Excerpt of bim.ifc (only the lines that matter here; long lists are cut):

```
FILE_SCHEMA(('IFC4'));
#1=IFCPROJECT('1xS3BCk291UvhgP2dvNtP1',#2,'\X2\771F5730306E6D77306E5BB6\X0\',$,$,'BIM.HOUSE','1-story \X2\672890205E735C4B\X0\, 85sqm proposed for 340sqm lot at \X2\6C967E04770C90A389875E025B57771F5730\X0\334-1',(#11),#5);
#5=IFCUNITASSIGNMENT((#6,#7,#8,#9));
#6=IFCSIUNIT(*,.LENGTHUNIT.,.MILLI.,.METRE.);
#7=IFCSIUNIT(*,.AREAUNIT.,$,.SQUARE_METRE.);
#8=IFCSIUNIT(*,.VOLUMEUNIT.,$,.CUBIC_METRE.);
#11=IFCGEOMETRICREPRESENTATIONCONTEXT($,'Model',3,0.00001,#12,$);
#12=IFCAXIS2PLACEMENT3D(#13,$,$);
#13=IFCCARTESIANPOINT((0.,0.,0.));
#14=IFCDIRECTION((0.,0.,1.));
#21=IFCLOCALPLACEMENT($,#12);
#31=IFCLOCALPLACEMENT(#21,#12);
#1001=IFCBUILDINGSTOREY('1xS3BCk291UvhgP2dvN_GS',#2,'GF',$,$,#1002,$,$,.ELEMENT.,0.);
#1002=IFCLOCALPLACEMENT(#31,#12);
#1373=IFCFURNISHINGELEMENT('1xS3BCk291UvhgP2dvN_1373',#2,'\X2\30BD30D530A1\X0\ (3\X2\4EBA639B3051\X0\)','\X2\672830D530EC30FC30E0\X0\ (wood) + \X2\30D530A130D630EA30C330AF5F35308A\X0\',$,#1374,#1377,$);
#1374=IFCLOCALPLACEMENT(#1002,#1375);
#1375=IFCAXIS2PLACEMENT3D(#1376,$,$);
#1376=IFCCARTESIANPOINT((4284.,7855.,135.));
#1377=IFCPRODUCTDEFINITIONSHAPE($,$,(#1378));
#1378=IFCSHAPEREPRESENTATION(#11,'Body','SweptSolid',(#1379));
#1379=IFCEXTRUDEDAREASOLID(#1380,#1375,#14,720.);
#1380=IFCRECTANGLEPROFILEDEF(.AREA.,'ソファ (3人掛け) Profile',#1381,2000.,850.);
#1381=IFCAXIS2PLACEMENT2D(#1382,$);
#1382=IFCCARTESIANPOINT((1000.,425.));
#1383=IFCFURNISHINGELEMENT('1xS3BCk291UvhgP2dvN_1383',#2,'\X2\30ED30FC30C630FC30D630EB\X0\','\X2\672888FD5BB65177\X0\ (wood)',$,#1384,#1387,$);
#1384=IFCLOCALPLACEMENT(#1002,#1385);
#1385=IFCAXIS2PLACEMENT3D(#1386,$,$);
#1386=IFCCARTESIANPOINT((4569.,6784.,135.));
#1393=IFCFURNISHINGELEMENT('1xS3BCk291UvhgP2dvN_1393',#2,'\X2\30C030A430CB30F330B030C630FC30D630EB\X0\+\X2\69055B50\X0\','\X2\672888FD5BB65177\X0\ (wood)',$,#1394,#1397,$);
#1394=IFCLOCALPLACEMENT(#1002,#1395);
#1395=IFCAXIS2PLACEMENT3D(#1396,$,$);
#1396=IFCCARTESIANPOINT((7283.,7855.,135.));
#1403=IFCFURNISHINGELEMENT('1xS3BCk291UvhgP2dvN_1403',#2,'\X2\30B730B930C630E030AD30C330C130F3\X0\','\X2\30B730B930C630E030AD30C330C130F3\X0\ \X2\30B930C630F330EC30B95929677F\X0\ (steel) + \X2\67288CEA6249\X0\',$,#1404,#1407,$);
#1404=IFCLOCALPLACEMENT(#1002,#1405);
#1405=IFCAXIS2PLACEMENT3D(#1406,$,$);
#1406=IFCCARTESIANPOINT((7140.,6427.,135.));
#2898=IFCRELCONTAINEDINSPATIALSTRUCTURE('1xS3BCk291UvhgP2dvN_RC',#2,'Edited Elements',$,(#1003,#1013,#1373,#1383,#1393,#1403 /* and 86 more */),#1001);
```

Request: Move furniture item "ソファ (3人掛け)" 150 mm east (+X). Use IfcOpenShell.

```python
import ifcopenshell
import ifcopenshell.api.geometry
import ifcopenshell.util.placement
import ifcopenshell.util.unit

model = ifcopenshell.open("bim.ifc")
unit_scale = ifcopenshell.util.unit.calculate_unit_scale(model)

item = model.by_id(1373)
matrix = ifcopenshell.util.placement.get_local_placement(item.ObjectPlacement)
matrix[0, 3] += 0.15 / unit_scale
ifcopenshell.api.geometry.edit_object_placement(model, product=item, matrix=matrix, is_si=False)

print(ifcopenshell.util.placement.get_local_placement(item.ObjectPlacement).round(3) + 0.0)

model.write("bim-out.ifc")
```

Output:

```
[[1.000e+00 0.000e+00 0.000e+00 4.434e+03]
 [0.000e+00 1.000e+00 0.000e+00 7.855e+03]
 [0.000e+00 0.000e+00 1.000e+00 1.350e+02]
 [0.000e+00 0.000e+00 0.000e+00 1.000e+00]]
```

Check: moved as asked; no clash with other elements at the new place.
